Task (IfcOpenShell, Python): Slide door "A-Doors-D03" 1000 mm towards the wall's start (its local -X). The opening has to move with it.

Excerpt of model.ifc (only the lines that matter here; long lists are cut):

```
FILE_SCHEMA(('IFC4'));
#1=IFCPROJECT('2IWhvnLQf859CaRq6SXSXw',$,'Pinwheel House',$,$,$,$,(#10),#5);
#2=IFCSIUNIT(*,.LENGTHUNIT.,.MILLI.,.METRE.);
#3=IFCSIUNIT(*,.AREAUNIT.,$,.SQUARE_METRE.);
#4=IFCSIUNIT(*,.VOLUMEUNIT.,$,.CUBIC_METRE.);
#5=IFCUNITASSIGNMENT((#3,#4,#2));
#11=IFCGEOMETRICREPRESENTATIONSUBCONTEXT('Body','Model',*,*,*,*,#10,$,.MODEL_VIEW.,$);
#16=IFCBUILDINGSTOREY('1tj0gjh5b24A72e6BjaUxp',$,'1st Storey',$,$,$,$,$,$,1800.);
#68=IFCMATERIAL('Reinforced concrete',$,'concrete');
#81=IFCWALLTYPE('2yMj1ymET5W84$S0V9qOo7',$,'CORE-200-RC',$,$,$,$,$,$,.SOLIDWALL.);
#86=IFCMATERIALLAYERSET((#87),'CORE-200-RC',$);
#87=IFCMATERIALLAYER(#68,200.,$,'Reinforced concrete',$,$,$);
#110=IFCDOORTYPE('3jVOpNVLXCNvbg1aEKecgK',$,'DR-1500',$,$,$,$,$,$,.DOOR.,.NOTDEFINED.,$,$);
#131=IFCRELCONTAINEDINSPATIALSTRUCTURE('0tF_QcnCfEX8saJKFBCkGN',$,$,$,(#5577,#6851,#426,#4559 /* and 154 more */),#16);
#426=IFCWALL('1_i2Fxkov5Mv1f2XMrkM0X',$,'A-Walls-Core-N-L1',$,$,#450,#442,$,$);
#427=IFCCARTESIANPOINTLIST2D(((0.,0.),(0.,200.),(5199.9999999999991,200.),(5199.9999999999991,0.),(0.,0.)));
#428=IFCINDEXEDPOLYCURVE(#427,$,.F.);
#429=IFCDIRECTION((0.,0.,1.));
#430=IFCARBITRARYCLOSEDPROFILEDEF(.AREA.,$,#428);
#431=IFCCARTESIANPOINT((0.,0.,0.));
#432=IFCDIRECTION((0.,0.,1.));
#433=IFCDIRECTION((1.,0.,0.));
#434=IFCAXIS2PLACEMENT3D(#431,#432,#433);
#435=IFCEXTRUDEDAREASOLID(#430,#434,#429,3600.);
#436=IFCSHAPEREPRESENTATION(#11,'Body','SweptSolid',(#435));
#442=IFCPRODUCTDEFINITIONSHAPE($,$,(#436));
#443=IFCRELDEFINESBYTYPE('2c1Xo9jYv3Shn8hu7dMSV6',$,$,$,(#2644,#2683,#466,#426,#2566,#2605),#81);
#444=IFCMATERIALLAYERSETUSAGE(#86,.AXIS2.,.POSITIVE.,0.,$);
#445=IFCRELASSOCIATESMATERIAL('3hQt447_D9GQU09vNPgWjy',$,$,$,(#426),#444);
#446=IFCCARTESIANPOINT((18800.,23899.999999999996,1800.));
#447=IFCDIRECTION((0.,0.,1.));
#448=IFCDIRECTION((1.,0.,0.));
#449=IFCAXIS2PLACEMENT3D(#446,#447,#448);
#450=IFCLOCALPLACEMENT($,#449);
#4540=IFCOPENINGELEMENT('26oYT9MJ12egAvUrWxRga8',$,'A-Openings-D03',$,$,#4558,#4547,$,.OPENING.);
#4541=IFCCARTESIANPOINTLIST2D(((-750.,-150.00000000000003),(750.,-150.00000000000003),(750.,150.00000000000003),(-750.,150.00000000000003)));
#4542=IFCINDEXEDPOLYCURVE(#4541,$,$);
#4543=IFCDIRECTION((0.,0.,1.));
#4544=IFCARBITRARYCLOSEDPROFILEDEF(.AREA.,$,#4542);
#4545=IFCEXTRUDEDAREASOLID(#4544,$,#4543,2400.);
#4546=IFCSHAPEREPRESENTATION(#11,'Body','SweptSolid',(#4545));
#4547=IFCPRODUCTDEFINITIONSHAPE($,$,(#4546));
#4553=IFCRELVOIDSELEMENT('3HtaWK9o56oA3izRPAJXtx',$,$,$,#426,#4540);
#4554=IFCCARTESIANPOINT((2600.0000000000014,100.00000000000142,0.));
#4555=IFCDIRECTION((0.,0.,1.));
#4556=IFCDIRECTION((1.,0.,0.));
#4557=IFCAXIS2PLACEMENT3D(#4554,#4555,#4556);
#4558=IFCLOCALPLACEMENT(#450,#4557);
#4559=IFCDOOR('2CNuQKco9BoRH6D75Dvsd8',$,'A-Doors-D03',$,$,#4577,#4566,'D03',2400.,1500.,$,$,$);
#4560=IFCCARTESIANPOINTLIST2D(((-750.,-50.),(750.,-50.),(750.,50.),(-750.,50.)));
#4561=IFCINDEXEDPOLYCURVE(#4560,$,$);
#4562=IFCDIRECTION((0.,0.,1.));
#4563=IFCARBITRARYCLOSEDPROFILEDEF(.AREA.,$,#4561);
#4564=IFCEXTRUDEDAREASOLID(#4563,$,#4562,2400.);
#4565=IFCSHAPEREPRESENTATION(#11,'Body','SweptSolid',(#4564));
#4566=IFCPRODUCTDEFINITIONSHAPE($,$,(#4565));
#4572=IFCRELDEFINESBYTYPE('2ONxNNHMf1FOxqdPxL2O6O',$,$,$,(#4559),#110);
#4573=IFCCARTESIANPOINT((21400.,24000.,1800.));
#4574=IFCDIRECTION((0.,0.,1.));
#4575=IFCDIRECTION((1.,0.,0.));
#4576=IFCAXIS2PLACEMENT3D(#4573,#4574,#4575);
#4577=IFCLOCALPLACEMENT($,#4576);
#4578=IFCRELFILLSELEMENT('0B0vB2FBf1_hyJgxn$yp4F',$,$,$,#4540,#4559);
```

```python
import ifcopenshell
import ifcopenshell.api.geometry
import ifcopenshell.util.placement
import ifcopenshell.util.unit

model = ifcopenshell.open("model.ifc")
unit_scale = ifcopenshell.util.unit.calculate_unit_scale(model)

door = model.by_guid("2CNuQKco9BoRH6D75Dvsd8")
opening = door.FillsVoids[0].RelatingOpeningElement
wall = opening.VoidsElements[0].RelatingBuildingElement

wall_matrix = ifcopenshell.util.placement.get_local_placement(wall.ObjectPlacement)
shift = wall_matrix[:3, 0] * -1 / unit_scale
before = ifcopenshell.util.placement.get_local_placement(door.ObjectPlacement)[:3, 3].copy()

# The door is not placed relative to its opening, so move both.
for product in (opening, door):
    matrix = ifcopenshell.util.placement.get_local_placement(product.ObjectPlacement)
    matrix[:3, 3] += shift
    ifcopenshell.api.geometry.edit_object_placement(model, product=product, matrix=matrix, is_si=False)

after = ifcopenshell.util.placement.get_local_placement(door.ObjectPlacement)[:3, 3]
print("door moved by", (after - before).round(3) + 0.0)

model.write("model_updated.ifc")
```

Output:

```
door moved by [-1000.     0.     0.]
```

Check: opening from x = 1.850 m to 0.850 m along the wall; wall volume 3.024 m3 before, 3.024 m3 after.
